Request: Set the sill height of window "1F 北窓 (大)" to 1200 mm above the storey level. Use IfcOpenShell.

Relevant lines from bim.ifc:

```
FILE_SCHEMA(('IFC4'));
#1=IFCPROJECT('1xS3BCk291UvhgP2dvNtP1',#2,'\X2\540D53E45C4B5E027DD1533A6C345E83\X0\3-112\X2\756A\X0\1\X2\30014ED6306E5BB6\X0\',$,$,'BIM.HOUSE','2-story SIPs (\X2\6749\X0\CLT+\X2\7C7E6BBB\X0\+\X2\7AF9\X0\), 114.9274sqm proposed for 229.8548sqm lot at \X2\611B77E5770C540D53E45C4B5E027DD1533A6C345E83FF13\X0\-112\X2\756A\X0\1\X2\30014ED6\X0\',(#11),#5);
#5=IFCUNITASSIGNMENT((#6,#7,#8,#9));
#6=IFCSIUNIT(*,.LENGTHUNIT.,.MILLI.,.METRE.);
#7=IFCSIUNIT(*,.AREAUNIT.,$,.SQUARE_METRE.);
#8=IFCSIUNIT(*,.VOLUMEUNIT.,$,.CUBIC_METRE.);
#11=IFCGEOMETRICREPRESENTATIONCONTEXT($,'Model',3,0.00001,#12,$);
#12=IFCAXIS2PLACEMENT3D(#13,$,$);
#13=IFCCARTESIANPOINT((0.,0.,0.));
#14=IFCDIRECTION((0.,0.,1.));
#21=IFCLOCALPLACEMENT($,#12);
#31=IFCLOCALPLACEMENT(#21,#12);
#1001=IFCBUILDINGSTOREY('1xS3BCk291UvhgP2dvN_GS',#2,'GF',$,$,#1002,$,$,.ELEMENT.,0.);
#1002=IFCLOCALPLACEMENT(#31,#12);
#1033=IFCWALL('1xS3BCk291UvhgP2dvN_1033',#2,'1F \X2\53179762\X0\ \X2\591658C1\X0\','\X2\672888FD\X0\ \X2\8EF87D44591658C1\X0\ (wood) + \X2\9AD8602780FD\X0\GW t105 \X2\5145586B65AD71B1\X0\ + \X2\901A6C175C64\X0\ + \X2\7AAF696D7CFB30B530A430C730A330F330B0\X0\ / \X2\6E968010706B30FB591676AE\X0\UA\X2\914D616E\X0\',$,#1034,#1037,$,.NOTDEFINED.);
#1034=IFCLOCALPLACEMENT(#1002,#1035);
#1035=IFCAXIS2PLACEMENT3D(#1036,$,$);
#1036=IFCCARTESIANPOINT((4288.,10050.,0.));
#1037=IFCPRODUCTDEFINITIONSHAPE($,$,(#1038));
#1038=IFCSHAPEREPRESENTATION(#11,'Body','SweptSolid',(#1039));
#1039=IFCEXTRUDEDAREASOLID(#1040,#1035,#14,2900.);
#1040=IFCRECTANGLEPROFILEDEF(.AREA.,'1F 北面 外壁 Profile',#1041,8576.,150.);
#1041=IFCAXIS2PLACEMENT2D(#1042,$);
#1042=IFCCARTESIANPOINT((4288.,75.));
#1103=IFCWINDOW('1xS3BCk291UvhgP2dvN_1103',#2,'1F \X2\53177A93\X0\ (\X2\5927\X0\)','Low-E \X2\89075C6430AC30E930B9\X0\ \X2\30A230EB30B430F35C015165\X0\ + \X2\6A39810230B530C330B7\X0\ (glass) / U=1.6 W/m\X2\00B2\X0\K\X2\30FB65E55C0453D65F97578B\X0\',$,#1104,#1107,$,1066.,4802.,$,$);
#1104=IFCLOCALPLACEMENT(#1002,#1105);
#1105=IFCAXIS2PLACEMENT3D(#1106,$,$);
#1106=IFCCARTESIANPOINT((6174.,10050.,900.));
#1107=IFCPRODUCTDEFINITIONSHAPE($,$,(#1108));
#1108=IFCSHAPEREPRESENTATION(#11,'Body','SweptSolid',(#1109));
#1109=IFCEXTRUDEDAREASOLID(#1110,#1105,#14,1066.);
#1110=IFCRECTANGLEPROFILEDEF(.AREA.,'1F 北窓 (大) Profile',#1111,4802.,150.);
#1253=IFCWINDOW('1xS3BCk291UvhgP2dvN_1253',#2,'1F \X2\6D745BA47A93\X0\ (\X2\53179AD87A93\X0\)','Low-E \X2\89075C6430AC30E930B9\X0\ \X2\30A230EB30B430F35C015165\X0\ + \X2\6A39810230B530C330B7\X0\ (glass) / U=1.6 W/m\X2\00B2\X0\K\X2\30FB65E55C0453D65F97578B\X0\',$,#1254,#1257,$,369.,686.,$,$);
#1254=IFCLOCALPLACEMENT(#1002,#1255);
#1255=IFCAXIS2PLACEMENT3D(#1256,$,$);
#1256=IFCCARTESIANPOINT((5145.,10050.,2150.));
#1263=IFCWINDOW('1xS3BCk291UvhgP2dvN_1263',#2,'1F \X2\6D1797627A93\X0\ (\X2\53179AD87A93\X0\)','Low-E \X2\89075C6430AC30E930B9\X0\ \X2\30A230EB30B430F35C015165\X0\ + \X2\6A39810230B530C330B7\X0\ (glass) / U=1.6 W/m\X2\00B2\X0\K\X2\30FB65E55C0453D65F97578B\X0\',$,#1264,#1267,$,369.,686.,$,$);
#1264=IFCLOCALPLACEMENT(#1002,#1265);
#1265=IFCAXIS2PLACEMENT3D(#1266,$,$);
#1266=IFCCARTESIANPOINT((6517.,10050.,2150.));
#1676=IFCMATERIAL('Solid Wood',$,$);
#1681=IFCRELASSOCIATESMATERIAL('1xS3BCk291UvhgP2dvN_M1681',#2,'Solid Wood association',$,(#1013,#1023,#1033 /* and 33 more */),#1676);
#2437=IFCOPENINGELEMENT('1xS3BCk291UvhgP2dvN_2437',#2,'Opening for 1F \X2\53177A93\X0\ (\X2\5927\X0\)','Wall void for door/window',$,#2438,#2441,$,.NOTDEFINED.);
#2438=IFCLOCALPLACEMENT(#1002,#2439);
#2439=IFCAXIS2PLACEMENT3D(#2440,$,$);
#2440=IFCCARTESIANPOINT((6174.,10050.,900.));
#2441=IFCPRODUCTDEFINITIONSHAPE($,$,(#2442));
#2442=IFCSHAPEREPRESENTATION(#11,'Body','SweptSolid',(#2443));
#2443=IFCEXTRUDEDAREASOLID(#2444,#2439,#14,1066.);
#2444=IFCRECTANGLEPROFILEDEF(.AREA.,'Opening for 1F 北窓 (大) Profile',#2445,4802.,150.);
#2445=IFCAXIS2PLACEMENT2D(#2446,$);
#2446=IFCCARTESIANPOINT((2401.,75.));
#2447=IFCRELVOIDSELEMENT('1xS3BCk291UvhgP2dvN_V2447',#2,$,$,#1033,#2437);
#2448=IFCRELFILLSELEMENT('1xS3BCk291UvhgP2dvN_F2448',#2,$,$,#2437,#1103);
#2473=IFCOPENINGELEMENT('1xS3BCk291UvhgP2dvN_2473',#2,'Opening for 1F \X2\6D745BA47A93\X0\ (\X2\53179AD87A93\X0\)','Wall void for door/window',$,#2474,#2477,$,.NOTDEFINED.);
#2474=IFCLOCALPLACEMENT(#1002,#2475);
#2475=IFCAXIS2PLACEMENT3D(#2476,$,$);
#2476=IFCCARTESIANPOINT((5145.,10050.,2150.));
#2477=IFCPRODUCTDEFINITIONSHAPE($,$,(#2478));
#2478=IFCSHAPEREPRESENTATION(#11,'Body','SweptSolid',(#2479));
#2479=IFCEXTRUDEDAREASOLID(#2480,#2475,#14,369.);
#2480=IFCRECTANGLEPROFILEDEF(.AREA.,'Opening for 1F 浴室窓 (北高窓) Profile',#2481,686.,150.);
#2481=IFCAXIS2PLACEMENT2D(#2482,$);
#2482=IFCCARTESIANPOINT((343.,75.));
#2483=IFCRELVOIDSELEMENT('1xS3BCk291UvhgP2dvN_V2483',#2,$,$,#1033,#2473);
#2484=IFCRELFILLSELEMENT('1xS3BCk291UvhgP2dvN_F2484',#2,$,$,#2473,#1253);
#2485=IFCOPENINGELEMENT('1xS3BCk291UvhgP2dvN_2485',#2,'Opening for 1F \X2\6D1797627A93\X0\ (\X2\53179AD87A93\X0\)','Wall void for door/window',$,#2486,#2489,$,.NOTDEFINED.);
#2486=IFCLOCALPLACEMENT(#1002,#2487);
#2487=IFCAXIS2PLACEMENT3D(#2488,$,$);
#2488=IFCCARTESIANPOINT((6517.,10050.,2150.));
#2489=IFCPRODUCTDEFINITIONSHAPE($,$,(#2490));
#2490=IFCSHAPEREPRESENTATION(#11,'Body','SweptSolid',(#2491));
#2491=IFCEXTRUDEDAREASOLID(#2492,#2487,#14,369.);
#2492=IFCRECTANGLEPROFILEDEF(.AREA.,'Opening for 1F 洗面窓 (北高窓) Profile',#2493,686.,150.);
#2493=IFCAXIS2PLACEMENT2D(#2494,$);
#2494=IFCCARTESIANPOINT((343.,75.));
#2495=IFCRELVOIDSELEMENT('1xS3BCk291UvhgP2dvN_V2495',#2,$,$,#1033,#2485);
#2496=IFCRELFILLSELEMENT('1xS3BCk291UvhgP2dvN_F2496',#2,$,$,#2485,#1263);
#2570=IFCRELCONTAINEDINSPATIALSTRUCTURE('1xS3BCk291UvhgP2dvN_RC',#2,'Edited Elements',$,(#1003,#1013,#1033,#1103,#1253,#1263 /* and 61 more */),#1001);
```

```python
import numpy as np
import ifcopenshell
import ifcopenshell.api.geometry
import ifcopenshell.geom
import ifcopenshell.util.element
import ifcopenshell.util.placement
import ifcopenshell.util.shape
import ifcopenshell.util.unit

model = ifcopenshell.open("bim.ifc")
unit_scale = ifcopenshell.util.unit.calculate_unit_scale(model)

window = model.by_guid("1xS3BCk291UvhgP2dvN_1103")
opening = window.FillsVoids[0].RelatingOpeningElement
storey = ifcopenshell.util.element.get_container(window, ifc_class="IfcBuildingStorey")
level = ifcopenshell.util.placement.get_local_placement(storey.ObjectPlacement)[2, 3]

# The opening's origin need not be at the sill, so measure its lowest point.
shape = ifcopenshell.geom.create_shape(ifcopenshell.geom.settings(), opening)
bottom = ifcopenshell.util.shape.get_shape_bottom_elevation(shape, shape.geometry) / unit_scale
dz = level + 1200.0 - bottom

shift = np.array([0.0, 0.0, dz])
# The window is not placed relative to its opening, so move both.
for product in (opening, window):
    matrix = ifcopenshell.util.placement.get_local_placement(product.ObjectPlacement)
    matrix[:3, 3] += shift
    ifcopenshell.api.geometry.edit_object_placement(model, product=product, matrix=matrix, is_si=False)

print(f"moved by {dz * unit_scale:+.3f} m")

model.write("bim_edited.ifc")
```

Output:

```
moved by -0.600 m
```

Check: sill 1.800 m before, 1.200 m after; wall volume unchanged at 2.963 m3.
